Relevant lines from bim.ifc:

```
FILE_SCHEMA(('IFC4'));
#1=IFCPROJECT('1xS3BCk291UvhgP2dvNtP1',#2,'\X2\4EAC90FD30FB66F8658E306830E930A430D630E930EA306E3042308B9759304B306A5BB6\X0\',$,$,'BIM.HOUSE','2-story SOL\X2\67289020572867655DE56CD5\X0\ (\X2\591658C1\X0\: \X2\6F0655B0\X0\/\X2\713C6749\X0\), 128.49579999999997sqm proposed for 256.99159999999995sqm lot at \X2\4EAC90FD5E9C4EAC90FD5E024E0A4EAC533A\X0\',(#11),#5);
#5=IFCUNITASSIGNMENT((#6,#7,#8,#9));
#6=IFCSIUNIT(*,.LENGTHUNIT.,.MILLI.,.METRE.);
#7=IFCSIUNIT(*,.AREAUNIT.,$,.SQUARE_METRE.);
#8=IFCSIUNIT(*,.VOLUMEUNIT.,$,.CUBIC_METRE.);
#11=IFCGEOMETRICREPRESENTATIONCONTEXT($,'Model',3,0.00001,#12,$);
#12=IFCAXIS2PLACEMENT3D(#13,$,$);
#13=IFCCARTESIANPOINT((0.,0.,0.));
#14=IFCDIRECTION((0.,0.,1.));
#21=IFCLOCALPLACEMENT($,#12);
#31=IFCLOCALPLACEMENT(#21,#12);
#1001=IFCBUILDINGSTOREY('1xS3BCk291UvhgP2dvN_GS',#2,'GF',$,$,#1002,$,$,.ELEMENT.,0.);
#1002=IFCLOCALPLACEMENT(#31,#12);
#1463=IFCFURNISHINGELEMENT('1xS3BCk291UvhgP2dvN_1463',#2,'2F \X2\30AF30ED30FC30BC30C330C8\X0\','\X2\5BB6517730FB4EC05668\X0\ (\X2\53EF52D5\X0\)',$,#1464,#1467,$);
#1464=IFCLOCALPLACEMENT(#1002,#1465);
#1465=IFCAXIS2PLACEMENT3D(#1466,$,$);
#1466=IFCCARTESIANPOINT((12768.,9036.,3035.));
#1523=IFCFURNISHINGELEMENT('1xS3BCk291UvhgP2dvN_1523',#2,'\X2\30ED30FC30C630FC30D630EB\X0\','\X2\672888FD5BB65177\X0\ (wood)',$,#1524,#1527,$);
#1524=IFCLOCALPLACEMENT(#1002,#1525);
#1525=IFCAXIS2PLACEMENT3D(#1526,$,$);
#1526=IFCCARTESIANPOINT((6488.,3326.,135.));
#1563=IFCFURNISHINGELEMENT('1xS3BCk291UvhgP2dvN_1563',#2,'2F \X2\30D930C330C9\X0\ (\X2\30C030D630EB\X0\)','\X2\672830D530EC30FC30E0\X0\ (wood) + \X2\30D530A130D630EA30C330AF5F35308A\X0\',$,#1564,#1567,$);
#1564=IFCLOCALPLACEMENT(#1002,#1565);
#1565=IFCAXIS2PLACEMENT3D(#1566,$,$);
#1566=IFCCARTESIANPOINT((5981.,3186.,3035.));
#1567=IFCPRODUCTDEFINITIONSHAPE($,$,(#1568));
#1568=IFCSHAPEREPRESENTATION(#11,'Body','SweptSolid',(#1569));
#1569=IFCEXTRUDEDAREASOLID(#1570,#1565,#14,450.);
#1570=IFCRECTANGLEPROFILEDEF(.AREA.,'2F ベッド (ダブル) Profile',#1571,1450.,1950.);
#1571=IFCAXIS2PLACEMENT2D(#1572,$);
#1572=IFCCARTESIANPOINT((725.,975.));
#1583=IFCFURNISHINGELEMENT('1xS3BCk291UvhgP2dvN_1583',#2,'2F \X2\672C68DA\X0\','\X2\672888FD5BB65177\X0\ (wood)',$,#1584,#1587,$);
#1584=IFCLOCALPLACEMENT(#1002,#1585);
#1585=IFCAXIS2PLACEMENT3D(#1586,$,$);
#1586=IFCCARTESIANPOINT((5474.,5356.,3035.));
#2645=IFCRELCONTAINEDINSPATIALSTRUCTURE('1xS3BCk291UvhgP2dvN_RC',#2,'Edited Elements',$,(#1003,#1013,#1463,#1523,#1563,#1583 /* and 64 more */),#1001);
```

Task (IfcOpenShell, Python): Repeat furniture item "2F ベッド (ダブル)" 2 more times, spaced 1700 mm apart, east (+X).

```python
import numpy as np
import ifcopenshell
import ifcopenshell.api.geometry
import ifcopenshell.api.root
import ifcopenshell.util.element
import ifcopenshell.util.placement
import ifcopenshell.util.unit

model = ifcopenshell.open("bim.ifc")
unit_scale = ifcopenshell.util.unit.calculate_unit_scale(model)


def reuse_history(source, copy):
    """copy_class also copies each property set's owner history, people and application; keep the originals."""
    for rel in copy.IsDefinedBy:
        if rel.is_a("IfcRelDefinesByProperties") and (history := rel.RelatingPropertyDefinition.OwnerHistory):
            rel.RelatingPropertyDefinition.OwnerHistory = source.OwnerHistory
            ifcopenshell.util.element.remove_deep2(model, history)


source = model.by_id(1563)
base = ifcopenshell.util.placement.get_local_placement(source.ObjectPlacement)
step = np.array([1.0, 0.0, 0.0]) * 1.7 / unit_scale

for i in range(1, 3):
    copy = ifcopenshell.api.root.copy_class(model, product=source)
    copy.Representation = ifcopenshell.util.element.copy_deep(
        model, source.Representation, exclude=["IfcGeometricRepresentationContext", "IfcRepresentationMap"]
    )
    reuse_history(source, copy)
    matrix = base.copy()
    matrix[:3, 3] += i * step
    print("added at", matrix[:3, 3].round(3) + 0.0)
    ifcopenshell.api.geometry.edit_object_placement(model, product=copy, matrix=matrix, is_si=False)

model.write("bim_edited.ifc")
```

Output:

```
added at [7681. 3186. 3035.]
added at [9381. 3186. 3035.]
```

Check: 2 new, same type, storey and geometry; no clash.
